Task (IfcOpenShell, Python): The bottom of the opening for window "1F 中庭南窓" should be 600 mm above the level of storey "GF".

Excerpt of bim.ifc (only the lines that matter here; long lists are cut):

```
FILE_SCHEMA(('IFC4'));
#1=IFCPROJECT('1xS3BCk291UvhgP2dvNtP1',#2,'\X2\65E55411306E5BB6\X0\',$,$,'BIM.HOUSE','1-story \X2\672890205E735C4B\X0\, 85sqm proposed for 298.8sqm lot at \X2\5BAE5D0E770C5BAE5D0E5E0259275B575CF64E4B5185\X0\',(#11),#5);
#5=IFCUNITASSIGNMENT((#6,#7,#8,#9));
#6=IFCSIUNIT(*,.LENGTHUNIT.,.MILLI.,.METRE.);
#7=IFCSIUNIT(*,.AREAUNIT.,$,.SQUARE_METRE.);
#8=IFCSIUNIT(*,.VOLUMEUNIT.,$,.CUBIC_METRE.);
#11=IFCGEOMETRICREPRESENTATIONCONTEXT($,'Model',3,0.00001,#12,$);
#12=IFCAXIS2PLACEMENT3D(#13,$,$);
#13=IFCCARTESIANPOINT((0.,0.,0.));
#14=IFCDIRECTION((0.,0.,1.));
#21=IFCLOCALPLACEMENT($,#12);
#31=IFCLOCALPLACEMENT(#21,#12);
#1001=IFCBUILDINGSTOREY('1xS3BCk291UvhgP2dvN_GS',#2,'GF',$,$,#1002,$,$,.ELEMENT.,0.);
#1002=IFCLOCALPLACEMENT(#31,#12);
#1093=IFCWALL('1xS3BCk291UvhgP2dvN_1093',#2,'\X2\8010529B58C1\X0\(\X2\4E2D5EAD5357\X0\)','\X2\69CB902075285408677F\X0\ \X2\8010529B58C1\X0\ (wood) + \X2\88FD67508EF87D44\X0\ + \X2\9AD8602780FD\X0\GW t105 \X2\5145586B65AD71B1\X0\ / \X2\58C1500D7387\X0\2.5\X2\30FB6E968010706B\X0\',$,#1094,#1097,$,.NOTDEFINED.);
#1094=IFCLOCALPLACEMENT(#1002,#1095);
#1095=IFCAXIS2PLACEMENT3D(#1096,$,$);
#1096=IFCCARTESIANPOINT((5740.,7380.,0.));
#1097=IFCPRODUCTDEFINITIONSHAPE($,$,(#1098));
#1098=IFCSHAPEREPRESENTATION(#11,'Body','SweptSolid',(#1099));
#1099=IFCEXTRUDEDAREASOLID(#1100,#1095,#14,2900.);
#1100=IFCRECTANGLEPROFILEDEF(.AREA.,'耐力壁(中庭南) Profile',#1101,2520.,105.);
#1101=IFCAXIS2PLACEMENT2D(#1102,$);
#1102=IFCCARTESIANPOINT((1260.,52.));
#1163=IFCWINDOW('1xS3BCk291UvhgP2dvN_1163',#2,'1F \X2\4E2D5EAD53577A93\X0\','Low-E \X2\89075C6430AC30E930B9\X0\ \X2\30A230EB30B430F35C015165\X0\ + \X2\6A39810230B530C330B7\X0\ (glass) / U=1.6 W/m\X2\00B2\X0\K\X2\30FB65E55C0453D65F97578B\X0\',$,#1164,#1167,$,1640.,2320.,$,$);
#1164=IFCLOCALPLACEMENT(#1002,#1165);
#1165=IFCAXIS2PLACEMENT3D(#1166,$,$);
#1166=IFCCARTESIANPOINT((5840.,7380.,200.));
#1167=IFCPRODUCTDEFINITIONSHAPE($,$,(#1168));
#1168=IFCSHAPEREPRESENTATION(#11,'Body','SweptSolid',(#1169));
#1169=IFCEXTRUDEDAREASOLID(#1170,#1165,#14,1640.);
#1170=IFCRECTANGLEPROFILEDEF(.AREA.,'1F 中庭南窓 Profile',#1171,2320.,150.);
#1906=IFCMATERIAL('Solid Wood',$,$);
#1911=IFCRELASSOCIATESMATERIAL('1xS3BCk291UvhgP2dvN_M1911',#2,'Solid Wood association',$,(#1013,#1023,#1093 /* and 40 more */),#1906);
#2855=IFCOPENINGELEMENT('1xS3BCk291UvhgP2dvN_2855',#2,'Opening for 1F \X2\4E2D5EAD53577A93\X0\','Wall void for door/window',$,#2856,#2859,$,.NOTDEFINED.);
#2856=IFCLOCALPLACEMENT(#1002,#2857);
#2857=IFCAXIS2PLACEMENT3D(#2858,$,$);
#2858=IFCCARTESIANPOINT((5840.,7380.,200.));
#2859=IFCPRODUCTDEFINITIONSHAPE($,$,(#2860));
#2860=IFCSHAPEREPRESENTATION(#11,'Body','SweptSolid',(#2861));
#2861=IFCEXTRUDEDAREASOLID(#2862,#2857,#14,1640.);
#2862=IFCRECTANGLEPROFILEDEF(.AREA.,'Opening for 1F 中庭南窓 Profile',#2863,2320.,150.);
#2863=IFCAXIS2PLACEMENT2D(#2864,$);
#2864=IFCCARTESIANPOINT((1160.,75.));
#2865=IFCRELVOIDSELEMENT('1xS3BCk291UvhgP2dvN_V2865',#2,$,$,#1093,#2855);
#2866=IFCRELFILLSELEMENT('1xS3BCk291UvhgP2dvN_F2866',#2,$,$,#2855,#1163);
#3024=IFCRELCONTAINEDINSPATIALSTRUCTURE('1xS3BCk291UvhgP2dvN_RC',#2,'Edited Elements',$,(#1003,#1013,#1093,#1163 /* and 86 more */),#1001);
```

```python
import numpy as np
import ifcopenshell
import ifcopenshell.api.geometry
import ifcopenshell.geom
import ifcopenshell.util.element
import ifcopenshell.util.placement
import ifcopenshell.util.shape
import ifcopenshell.util.unit

model = ifcopenshell.open("bim.ifc")
unit_scale = ifcopenshell.util.unit.calculate_unit_scale(model)

window = model.by_id(1163)
opening = window.FillsVoids[0].RelatingOpeningElement
storey = ifcopenshell.util.element.get_container(window, ifc_class="IfcBuildingStorey")
level = ifcopenshell.util.placement.get_local_placement(storey.ObjectPlacement)[2, 3]

# The opening's origin need not be at the sill, so measure its lowest point.
shape = ifcopenshell.geom.create_shape(ifcopenshell.geom.settings(), opening)
bottom = ifcopenshell.util.shape.get_shape_bottom_elevation(shape, shape.geometry) / unit_scale
dz = level + 0.6 / unit_scale - bottom

shift = np.array([0.0, 0.0, dz])
# The window is not placed relative to its opening, so move both.
for product in (opening, window):
    matrix = ifcopenshell.util.placement.get_local_placement(product.ObjectPlacement)
    matrix[:3, 3] += shift
    ifcopenshell.api.geometry.edit_object_placement(model, product=product, matrix=matrix, is_si=False)

print(f"moved by {dz * unit_scale:+.3f} m")

model.write("bim_updated.ifc")
```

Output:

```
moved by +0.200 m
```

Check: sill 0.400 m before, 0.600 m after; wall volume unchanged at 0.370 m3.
